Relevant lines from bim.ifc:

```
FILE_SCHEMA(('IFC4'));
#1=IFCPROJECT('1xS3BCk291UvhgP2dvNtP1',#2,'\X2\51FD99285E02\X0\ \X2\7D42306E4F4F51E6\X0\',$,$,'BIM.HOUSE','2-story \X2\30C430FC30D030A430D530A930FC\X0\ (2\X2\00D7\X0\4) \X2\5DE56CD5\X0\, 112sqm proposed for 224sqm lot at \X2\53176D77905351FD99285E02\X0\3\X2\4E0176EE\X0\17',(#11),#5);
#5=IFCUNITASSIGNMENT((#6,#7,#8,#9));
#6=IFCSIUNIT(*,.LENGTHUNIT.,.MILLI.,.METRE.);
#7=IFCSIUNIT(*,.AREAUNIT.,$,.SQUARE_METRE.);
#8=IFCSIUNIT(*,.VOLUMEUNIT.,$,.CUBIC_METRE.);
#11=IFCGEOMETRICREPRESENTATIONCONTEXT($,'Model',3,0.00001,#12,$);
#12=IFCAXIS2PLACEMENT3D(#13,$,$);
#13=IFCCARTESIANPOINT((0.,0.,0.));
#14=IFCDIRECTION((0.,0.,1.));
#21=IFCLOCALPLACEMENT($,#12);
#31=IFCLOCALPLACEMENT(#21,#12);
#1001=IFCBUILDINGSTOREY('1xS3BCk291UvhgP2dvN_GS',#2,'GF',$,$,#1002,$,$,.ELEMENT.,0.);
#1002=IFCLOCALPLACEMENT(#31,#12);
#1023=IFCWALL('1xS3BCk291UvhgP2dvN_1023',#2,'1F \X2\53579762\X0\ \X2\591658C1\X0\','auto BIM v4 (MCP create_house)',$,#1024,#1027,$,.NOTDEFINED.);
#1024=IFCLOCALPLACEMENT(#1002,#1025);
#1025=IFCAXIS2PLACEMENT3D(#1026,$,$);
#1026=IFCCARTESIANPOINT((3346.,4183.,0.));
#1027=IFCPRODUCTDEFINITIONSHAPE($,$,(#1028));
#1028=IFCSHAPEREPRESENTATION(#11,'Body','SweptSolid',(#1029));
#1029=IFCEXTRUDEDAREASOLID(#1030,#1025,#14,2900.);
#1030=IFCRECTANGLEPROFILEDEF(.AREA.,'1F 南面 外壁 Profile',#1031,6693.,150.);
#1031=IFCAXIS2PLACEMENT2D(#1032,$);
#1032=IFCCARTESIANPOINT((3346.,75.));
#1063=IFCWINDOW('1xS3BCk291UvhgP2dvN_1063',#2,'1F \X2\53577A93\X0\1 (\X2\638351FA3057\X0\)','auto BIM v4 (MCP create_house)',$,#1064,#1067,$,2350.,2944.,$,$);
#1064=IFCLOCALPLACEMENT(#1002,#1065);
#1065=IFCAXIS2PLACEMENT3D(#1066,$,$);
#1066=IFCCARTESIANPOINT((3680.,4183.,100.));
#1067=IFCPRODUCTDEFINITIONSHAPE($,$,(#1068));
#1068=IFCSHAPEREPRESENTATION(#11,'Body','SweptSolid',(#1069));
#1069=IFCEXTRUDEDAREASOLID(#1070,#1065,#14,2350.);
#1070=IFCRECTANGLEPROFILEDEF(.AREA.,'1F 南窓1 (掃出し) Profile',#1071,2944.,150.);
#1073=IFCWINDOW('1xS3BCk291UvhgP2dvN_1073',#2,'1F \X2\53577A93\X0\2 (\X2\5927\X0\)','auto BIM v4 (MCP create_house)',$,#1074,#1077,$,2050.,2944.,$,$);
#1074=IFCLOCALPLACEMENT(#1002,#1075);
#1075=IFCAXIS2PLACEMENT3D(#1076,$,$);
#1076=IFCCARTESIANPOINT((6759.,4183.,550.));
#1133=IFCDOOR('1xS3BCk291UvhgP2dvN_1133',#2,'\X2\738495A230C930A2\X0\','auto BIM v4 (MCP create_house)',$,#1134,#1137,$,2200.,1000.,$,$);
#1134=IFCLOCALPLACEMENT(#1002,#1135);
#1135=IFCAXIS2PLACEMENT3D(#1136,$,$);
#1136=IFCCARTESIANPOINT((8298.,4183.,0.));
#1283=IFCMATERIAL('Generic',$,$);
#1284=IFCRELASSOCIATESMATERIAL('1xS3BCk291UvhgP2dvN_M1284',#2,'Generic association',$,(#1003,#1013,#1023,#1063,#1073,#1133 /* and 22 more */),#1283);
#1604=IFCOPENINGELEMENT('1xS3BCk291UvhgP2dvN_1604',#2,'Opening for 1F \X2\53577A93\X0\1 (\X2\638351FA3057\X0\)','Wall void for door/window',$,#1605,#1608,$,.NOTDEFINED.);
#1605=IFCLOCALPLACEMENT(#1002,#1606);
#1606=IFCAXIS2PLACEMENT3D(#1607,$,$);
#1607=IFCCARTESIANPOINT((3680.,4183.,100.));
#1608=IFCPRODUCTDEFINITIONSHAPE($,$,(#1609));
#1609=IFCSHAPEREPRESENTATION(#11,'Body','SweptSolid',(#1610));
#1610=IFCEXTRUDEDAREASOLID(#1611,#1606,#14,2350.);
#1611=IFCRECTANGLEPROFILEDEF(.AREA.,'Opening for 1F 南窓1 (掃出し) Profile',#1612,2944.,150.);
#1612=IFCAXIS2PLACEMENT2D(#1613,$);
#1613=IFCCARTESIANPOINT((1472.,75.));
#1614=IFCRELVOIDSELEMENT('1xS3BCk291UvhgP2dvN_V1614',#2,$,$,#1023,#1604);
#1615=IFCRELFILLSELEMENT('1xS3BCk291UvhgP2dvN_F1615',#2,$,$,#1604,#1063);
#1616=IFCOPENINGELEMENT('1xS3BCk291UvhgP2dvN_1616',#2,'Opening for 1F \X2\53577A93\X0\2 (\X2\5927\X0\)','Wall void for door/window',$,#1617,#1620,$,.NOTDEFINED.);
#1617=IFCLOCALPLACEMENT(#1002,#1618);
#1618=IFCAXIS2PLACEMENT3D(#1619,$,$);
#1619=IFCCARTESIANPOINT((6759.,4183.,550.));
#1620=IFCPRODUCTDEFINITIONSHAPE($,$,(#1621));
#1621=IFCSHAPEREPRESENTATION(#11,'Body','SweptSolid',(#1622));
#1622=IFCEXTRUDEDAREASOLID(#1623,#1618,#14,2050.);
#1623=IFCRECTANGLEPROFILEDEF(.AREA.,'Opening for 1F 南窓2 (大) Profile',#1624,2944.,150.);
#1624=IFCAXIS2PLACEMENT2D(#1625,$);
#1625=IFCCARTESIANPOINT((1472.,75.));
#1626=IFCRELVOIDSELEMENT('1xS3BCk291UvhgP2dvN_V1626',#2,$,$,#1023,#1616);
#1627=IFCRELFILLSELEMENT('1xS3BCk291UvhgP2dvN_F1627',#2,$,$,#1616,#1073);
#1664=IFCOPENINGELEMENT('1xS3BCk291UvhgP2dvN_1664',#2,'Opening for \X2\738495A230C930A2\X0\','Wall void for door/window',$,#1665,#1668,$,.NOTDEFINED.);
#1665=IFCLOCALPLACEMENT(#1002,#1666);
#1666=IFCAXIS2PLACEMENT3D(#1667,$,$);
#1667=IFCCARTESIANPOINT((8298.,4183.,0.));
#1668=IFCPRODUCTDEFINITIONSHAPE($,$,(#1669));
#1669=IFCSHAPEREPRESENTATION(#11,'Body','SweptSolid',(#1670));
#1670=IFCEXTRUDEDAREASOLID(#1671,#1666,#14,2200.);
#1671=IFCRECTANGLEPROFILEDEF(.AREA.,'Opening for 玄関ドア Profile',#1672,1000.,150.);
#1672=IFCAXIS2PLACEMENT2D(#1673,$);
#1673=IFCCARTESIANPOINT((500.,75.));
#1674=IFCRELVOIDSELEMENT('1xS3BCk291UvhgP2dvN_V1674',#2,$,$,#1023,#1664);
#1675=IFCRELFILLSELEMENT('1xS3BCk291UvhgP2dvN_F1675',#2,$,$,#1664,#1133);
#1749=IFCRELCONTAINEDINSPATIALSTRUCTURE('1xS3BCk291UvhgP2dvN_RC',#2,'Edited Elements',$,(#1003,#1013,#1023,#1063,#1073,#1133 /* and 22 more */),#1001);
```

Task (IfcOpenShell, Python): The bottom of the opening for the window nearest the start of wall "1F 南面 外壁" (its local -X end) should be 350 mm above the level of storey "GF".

```python
import numpy as np
import ifcopenshell
import ifcopenshell.api.geometry
import ifcopenshell.geom
import ifcopenshell.util.element
import ifcopenshell.util.placement
import ifcopenshell.util.shape
import ifcopenshell.util.unit

model = ifcopenshell.open("bim.ifc")
unit_scale = ifcopenshell.util.unit.calculate_unit_scale(model)

window = model.by_guid("1xS3BCk291UvhgP2dvN_1063")
opening = window.FillsVoids[0].RelatingOpeningElement
storey = ifcopenshell.util.element.get_container(window, ifc_class="IfcBuildingStorey")
level = ifcopenshell.util.placement.get_local_placement(storey.ObjectPlacement)[2, 3]

# The opening's origin need not be at the sill, so measure its lowest point.
shape = ifcopenshell.geom.create_shape(ifcopenshell.geom.settings(), opening)
bottom = ifcopenshell.util.shape.get_shape_bottom_elevation(shape, shape.geometry) / unit_scale
dz = level + 350.0 - bottom

shift = np.array([0.0, 0.0, dz])
# The window is not placed relative to its opening, so move both.
for product in (opening, window):
    matrix = ifcopenshell.util.placement.get_local_placement(product.ObjectPlacement)
    matrix[:3, 3] += shift
    ifcopenshell.api.geometry.edit_object_placement(model, product=product, matrix=matrix, is_si=False)

print(f"moved by {dz * unit_scale:+.3f} m")

model.write("bim_rev.ifc")
```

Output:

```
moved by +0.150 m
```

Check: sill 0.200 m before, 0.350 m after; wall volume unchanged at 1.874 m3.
